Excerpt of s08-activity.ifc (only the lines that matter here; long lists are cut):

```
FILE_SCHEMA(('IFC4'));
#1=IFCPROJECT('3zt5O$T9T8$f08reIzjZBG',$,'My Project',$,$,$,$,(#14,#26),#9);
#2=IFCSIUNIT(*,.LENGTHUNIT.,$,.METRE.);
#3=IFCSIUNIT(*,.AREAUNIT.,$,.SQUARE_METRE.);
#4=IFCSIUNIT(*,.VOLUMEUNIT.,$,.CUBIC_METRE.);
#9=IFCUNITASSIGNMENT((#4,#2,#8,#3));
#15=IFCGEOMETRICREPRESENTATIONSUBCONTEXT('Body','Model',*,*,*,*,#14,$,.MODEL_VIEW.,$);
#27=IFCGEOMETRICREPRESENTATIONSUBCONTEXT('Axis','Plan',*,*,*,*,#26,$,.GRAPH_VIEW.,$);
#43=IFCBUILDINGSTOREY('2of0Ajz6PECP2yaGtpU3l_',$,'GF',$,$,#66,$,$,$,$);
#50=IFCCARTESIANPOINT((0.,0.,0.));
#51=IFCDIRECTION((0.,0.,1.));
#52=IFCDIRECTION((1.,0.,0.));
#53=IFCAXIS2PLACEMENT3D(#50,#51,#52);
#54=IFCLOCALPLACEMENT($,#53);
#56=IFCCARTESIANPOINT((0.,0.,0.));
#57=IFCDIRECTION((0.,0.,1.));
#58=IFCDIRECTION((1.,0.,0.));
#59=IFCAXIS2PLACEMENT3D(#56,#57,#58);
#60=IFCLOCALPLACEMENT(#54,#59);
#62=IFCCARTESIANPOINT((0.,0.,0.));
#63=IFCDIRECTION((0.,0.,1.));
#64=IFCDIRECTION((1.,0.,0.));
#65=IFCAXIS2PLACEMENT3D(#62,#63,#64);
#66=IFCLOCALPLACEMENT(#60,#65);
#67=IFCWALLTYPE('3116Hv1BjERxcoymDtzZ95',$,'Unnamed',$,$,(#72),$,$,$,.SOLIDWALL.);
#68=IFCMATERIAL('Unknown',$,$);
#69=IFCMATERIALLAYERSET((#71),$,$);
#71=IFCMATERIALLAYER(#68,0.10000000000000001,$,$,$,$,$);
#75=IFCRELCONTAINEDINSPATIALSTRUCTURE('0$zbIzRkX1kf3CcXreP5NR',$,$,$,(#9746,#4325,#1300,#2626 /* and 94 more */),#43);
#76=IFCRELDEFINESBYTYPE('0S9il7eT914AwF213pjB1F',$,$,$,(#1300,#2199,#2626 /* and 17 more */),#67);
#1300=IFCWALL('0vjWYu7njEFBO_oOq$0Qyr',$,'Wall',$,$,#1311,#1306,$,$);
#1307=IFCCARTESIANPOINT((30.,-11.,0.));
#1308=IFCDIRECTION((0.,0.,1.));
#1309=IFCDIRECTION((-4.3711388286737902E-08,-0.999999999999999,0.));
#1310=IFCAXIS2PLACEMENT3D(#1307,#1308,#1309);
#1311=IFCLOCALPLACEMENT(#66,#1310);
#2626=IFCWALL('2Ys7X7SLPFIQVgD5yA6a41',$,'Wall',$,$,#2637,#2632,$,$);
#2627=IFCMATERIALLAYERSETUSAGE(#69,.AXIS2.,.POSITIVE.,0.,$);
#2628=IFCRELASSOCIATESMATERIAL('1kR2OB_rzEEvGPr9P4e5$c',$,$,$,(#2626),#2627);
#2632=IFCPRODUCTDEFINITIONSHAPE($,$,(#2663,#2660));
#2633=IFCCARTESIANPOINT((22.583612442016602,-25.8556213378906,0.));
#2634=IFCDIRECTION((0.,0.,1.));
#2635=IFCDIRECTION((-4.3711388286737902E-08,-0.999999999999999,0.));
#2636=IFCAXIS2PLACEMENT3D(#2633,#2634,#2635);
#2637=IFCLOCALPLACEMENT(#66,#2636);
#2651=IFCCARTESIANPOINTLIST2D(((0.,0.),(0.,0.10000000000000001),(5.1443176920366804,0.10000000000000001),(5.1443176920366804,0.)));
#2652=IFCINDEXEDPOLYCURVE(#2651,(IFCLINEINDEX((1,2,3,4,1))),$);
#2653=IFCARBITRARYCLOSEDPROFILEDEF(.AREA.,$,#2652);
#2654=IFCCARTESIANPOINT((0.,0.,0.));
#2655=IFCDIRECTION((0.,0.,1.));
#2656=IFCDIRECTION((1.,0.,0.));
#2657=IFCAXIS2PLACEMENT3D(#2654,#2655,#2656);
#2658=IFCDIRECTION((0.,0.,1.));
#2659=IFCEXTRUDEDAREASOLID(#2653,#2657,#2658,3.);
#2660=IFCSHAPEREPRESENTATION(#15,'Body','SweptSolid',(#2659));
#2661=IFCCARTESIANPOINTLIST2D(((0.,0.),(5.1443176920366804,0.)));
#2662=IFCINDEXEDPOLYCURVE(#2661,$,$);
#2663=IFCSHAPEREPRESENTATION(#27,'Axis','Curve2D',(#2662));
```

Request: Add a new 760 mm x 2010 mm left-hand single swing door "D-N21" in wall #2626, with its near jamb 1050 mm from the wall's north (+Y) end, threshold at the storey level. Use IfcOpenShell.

```python
import numpy as np
import ifcopenshell
import ifcopenshell.api.feature
import ifcopenshell.api.geometry
import ifcopenshell.api.root
import ifcopenshell.api.spatial
import ifcopenshell.geom
import ifcopenshell.util.element
import ifcopenshell.util.placement
import ifcopenshell.util.representation
import ifcopenshell.util.shape
import ifcopenshell.util.unit

model = ifcopenshell.open("s08-activity.ifc")
unit_scale = ifcopenshell.util.unit.calculate_unit_scale(model)
settings = ifcopenshell.geom.settings()


def volume(element):
    """Net volume in cubic metres, openings subtracted."""
    shape = ifcopenshell.geom.create_shape(settings, element)
    return ifcopenshell.util.shape.get_volume(shape.geometry)


wall = model.by_guid("2Ys7X7SLPFIQVgD5yA6a41")
storey = ifcopenshell.util.element.get_container(wall, ifc_class="IfcBuildingStorey")
context = ifcopenshell.util.representation.get_context(model, "Model", "Body", "MODEL_VIEW")
before = volume(wall)

width, height, from_end, sill = 0.76, 2.01, 1.05, 0.0  # metres

# The wall runs along its own X axis, and the end named is its -X end.
wall_shape = ifcopenshell.geom.create_shape(settings, wall)
x, y, z = ifcopenshell.util.shape.get_vertices(wall_shape.geometry).T
start = x.min() + from_end
face, thickness = float(y.min()), float(y.max() - y.min())
wall_matrix = ifcopenshell.util.placement.get_local_placement(wall.ObjectPlacement)
level = ifcopenshell.util.placement.get_local_placement(storey.ObjectPlacement)[2, 3]


def in_wall(x, y):
    """Placement at x, y metres in the wall's axes, at sill height."""
    matrix = wall_matrix.copy()
    matrix[:, 3] = wall_matrix @ np.array([x / unit_scale, y / unit_scale, 0.0, 1.0])
    matrix[2, 3] = level + sill / unit_scale
    return matrix


# Opening: a box that overshoots both wall faces by 50 mm.
opening = ifcopenshell.api.root.create_entity(model, ifc_class="IfcOpeningElement", predefined_type="OPENING")
box = ifcopenshell.api.geometry.add_wall_representation(
    model, context=context, length=width, height=height, thickness=thickness + 0.1
)
ifcopenshell.api.geometry.assign_representation(model, product=opening, representation=box)
ifcopenshell.api.geometry.edit_object_placement(model, product=opening, matrix=in_wall(start, face - 0.05), is_si=False)
ifcopenshell.api.feature.add_feature(model, feature=opening, element=wall)

door = ifcopenshell.api.root.create_entity(model, ifc_class="IfcDoor", name="D-N21", predefined_type="DOOR")
door.OverallWidth, door.OverallHeight = width / unit_scale, height / unit_scale
door.OperationType = "SINGLE_SWING_LEFT"
body = ifcopenshell.api.geometry.add_door_representation(
    model,
    context=context,
    overall_width=door.OverallWidth,
    overall_height=door.OverallHeight,
    operation_type="SINGLE_SWING_LEFT",
    lining_properties={"LiningDepth": thickness / unit_scale, "ThresholdDepth": thickness / unit_scale},
)
ifcopenshell.api.geometry.assign_representation(model, product=door, representation=body)
ifcopenshell.api.spatial.assign_container(model, products=[door], relating_structure=storey)
ifcopenshell.api.feature.add_filling(model, opening=opening, element=door)

# The lining spans the wall, so the door starts at the wall face.
ifcopenshell.api.geometry.edit_object_placement(model, product=door, matrix=in_wall(start, face), is_si=False)

after = volume(wall)

print(f"wall volume {before:.3f} -> {after:.3f} m3")

model.write("s08-activity_v2.ifc")
```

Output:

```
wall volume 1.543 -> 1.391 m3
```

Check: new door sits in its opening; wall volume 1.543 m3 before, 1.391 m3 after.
